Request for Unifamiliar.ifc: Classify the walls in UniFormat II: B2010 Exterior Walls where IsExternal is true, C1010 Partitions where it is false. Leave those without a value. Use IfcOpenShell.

First a look at what the model holds.

```python
import ifcopenshell
import ifcopenshell.util.element

model = ifcopenshell.open("Unifamiliar.ifc")
print(model.schema)
print("classifications:", [c.Name for c in model.by_type("IfcClassification")])
values = [ifcopenshell.util.element.get_pset(e, "Pset_WallCommon", "IsExternal") for e in model.by_type("IfcWall")]
for value in (True, False, None):
    print("IsExternal", value, values.count(value))
```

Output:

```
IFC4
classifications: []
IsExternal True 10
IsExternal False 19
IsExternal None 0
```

```python
import ifcopenshell
import ifcopenshell.api.classification
import ifcopenshell.util.element

model = ifcopenshell.open("Unifamiliar.ifc")

system = ifcopenshell.api.classification.add_classification(model, classification="UniFormat II")

walls = model.by_type("IfcWall")
external = {e: ifcopenshell.util.element.get_pset(e, "Pset_WallCommon", "IsExternal") for e in walls}
for flag, code, name in ((True, "B2010", "Exterior Walls"), (False, "C1010", "Partitions")):
    products = [e for e in walls if external[e] is flag]
    ifcopenshell.api.classification.add_reference(
        model, products=products, classification=system, identification=code, name=name
    )
    print(code, len(products))

model.write("Unifamiliar_updated.ifc")
```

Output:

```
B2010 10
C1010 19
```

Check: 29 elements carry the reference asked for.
